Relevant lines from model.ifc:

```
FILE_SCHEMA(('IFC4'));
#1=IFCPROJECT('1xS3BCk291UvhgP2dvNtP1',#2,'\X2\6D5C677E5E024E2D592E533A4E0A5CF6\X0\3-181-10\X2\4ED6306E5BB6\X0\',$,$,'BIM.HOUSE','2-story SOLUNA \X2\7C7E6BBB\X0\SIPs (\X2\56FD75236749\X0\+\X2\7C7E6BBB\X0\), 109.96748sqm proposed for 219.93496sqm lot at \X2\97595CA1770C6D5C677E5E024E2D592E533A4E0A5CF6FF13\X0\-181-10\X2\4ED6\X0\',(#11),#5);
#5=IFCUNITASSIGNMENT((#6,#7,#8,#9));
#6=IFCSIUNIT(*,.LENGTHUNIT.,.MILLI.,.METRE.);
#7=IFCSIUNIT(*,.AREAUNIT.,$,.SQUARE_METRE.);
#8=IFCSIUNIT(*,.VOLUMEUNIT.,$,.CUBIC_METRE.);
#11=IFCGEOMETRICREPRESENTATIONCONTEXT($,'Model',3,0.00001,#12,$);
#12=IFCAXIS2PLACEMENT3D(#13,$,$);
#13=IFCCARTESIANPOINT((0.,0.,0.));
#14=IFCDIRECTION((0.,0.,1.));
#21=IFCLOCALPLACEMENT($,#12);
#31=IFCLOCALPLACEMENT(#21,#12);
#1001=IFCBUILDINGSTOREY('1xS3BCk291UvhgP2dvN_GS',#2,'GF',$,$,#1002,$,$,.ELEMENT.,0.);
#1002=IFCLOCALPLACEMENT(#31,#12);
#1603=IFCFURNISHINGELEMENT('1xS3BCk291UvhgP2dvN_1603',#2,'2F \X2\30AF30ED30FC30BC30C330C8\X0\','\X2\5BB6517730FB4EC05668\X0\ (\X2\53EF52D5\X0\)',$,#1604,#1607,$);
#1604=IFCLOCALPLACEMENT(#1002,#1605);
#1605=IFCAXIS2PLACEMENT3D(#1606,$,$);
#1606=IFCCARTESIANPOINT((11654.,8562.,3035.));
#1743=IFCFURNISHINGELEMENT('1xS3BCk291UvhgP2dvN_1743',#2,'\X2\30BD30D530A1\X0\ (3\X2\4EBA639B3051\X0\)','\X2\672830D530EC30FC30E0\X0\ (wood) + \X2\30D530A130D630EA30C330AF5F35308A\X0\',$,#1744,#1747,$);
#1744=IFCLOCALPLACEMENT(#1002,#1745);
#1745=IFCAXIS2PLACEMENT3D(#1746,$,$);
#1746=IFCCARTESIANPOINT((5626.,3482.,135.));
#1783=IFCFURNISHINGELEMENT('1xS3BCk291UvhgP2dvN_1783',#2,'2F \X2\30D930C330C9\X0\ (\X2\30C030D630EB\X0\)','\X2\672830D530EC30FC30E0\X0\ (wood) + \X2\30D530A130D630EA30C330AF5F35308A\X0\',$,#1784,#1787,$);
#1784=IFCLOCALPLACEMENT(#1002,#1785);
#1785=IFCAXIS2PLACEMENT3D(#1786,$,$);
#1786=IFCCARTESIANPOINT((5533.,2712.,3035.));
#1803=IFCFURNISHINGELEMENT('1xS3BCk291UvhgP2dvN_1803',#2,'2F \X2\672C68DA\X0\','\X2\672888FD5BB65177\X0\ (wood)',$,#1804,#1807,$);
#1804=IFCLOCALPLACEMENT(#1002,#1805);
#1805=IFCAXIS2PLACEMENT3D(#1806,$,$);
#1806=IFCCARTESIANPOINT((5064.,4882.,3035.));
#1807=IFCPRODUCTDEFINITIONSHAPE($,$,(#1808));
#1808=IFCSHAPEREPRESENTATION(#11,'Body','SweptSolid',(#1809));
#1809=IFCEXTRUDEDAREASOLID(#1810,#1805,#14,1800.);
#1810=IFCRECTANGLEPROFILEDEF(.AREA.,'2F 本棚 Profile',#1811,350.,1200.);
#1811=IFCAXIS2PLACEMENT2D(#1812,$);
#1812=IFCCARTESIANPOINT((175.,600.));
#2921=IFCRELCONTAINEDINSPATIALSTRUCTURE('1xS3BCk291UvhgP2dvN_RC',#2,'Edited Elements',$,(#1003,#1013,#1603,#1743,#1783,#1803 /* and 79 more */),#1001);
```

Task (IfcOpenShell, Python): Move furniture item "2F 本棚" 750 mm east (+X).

```python
import ifcopenshell
import ifcopenshell.api.geometry
import ifcopenshell.util.placement
import ifcopenshell.util.unit

model = ifcopenshell.open("model.ifc")
unit_scale = ifcopenshell.util.unit.calculate_unit_scale(model)

item = model.by_id(1803)
matrix = ifcopenshell.util.placement.get_local_placement(item.ObjectPlacement)
matrix[0, 3] += 0.75 / unit_scale
ifcopenshell.api.geometry.edit_object_placement(model, product=item, matrix=matrix, is_si=False)

print(ifcopenshell.util.placement.get_local_placement(item.ObjectPlacement).round(3) + 0.0)

model.write("model-out.ifc")
```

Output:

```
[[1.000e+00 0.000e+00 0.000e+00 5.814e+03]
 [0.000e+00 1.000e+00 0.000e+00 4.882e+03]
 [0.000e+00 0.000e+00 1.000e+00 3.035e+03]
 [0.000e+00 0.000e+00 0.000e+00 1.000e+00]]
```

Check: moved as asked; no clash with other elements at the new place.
